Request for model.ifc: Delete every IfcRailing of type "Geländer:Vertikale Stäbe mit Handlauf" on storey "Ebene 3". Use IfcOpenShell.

First a look at what the model holds.

```python
import ifcopenshell
import ifcopenshell.util.element

model = ifcopenshell.open("model.ifc")
print(model.schema)
storey = next(s for s in model.by_type("IfcBuildingStorey") if s.Name == "Ebene 3")
railings = [e for e in ifcopenshell.util.element.get_decomposition(storey) if e.is_a("IfcRailing")]
seen = {}
for e in railings:
    element_type = ifcopenshell.util.element.get_type(e)
    name = element_type.Name if element_type not in (None, e) else None
    seen[name] = seen.get(name, 0) + 1
for name, count in sorted(seen.items(), key=str):
    print(count, "x", name)
```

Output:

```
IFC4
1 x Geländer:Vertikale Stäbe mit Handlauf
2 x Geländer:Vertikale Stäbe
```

```python
import ifcopenshell
import ifcopenshell.api.root
import ifcopenshell.util.element

model = ifcopenshell.open("model.ifc")

storey = next(s for s in model.by_type("IfcBuildingStorey") if s.Name == "Ebene 3")
railings = [e for e in ifcopenshell.util.element.get_decomposition(storey) if e.is_a("IfcRailing")]
targets = [e for e in railings if (t := ifcopenshell.util.element.get_type(e)) not in (None, e) and t.Name == "Geländer:Vertikale Stäbe mit Handlauf"]

for e in targets:
    ifcopenshell.api.root.remove_product(model, product=e)
print(len(targets), "removed")

model.write("model_v2.ifc")
```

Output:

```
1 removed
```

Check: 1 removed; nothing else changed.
